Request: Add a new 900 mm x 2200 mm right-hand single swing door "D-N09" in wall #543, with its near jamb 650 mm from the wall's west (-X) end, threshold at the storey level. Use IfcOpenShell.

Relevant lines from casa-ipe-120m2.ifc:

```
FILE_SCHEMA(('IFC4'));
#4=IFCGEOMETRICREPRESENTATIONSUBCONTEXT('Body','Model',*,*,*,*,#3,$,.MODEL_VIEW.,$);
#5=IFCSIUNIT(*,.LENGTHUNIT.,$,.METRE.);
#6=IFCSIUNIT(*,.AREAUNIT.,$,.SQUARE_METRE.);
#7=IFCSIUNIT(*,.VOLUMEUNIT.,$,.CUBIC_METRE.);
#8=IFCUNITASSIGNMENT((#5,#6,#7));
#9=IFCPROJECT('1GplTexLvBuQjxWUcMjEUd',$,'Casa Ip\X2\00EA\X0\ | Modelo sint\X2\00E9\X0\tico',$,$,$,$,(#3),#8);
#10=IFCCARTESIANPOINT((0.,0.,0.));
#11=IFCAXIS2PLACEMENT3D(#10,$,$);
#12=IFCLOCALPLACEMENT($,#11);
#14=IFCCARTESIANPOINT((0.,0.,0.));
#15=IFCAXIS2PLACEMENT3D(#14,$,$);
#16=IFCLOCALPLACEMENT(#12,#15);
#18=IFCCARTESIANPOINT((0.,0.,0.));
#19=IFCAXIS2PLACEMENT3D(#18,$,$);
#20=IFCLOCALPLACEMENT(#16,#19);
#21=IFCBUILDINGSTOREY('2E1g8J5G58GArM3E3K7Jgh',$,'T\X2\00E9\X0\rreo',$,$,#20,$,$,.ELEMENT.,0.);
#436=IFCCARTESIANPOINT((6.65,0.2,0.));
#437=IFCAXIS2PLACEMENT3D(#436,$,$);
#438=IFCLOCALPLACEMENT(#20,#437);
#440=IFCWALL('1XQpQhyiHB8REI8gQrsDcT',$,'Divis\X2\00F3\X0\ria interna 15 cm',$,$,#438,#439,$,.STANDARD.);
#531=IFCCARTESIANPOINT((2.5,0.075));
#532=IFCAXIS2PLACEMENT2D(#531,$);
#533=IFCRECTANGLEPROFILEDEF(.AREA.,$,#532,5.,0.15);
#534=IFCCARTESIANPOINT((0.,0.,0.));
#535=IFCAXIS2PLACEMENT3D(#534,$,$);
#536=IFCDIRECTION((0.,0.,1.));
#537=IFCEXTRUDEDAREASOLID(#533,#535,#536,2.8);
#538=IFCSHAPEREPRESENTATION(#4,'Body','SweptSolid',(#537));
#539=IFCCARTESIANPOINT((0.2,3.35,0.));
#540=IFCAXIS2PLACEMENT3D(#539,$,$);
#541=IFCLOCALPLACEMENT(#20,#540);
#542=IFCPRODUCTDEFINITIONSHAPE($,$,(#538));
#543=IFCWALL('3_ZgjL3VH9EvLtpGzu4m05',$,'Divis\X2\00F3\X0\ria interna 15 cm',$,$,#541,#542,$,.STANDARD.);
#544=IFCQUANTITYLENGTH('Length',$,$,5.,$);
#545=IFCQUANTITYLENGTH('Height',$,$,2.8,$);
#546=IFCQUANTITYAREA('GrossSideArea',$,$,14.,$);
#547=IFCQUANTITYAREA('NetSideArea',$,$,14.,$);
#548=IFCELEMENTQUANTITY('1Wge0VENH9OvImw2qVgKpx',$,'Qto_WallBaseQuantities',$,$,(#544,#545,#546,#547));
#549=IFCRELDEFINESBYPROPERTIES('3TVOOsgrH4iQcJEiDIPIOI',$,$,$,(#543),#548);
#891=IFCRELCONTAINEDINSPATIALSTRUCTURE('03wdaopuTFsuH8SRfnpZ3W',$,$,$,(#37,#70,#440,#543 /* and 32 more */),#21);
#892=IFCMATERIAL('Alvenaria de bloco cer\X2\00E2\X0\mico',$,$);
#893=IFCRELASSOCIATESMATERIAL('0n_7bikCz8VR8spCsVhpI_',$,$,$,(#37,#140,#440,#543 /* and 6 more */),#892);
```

```python
import numpy as np
import ifcopenshell
import ifcopenshell.api.feature
import ifcopenshell.api.geometry
import ifcopenshell.api.pset
import ifcopenshell.api.root
import ifcopenshell.api.spatial
import ifcopenshell.geom
import ifcopenshell.util.element
import ifcopenshell.util.placement
import ifcopenshell.util.representation
import ifcopenshell.util.shape
import ifcopenshell.util.unit

model = ifcopenshell.open("casa-ipe-120m2.ifc")
unit_scale = ifcopenshell.util.unit.calculate_unit_scale(model)
area_scale = ifcopenshell.util.unit.calculate_unit_scale(model, "AREAUNIT")
settings = ifcopenshell.geom.settings()


def volume(element):
    """Net volume in cubic metres, openings subtracted."""
    shape = ifcopenshell.geom.create_shape(settings, element)
    return ifcopenshell.util.shape.get_volume(shape.geometry)


wall = model.by_guid("3_ZgjL3VH9EvLtpGzu4m05")
storey = ifcopenshell.util.element.get_container(wall, ifc_class="IfcBuildingStorey")
context = ifcopenshell.util.representation.get_context(model, "Model", "Body", "MODEL_VIEW")
before = volume(wall)

width, height, from_end, sill = 0.9, 2.2, 0.65, 0.0  # metres

# The wall runs along its own X axis, and the end named is its -X end.
wall_shape = ifcopenshell.geom.create_shape(settings, wall)
x, y, z = ifcopenshell.util.shape.get_vertices(wall_shape.geometry).T
start = x.min() + from_end
face, thickness = float(y.min()), float(y.max() - y.min())
wall_matrix = ifcopenshell.util.placement.get_local_placement(wall.ObjectPlacement)
level = ifcopenshell.util.placement.get_local_placement(storey.ObjectPlacement)[2, 3]


def in_wall(x, y):
    """Placement at x, y metres in the wall's axes, at sill height."""
    matrix = wall_matrix.copy()
    matrix[:, 3] = wall_matrix @ np.array([x / unit_scale, y / unit_scale, 0.0, 1.0])
    matrix[2, 3] = level + sill / unit_scale
    return matrix


# Opening: a box that overshoots both wall faces by 50 mm.
opening = ifcopenshell.api.root.create_entity(model, ifc_class="IfcOpeningElement", predefined_type="OPENING")
box = ifcopenshell.api.geometry.add_wall_representation(
    model, context=context, length=width, height=height, thickness=thickness + 0.1
)
ifcopenshell.api.geometry.assign_representation(model, product=opening, representation=box)
ifcopenshell.api.geometry.edit_object_placement(model, product=opening, matrix=in_wall(start, face - 0.05), is_si=False)
ifcopenshell.api.feature.add_feature(model, feature=opening, element=wall)

door = ifcopenshell.api.root.create_entity(model, ifc_class="IfcDoor", name="D-N09", predefined_type="DOOR")
door.OverallWidth, door.OverallHeight = width / unit_scale, height / unit_scale
door.OperationType = "SINGLE_SWING_RIGHT"
body = ifcopenshell.api.geometry.add_door_representation(
    model,
    context=context,
    overall_width=door.OverallWidth,
    overall_height=door.OverallHeight,
    operation_type="SINGLE_SWING_RIGHT",
    lining_properties={"LiningDepth": thickness / unit_scale, "ThresholdDepth": thickness / unit_scale},
)
ifcopenshell.api.geometry.assign_representation(model, product=door, representation=body)
ifcopenshell.api.spatial.assign_container(model, products=[door], relating_structure=storey)
ifcopenshell.api.feature.add_filling(model, opening=opening, element=door)

# The lining spans the wall, so the door starts at the wall face.
ifcopenshell.api.geometry.edit_object_placement(model, product=door, matrix=in_wall(start, face), is_si=False)

after = volume(wall)

# Update the wall's stored quantities.
qto = model.by_id(ifcopenshell.util.element.get_pset(wall, "Qto_WallBaseQuantities", should_inherit=False)["id"])
ifcopenshell.api.pset.edit_qto(model, qto=qto, properties={"NetSideArea": after / thickness / area_scale})

print(f"wall volume {before:.3f} -> {after:.3f} m3")

model.write("casa-ipe-120m2_updated.ifc")
```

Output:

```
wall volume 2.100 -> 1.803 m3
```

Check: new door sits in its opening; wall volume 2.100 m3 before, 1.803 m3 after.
